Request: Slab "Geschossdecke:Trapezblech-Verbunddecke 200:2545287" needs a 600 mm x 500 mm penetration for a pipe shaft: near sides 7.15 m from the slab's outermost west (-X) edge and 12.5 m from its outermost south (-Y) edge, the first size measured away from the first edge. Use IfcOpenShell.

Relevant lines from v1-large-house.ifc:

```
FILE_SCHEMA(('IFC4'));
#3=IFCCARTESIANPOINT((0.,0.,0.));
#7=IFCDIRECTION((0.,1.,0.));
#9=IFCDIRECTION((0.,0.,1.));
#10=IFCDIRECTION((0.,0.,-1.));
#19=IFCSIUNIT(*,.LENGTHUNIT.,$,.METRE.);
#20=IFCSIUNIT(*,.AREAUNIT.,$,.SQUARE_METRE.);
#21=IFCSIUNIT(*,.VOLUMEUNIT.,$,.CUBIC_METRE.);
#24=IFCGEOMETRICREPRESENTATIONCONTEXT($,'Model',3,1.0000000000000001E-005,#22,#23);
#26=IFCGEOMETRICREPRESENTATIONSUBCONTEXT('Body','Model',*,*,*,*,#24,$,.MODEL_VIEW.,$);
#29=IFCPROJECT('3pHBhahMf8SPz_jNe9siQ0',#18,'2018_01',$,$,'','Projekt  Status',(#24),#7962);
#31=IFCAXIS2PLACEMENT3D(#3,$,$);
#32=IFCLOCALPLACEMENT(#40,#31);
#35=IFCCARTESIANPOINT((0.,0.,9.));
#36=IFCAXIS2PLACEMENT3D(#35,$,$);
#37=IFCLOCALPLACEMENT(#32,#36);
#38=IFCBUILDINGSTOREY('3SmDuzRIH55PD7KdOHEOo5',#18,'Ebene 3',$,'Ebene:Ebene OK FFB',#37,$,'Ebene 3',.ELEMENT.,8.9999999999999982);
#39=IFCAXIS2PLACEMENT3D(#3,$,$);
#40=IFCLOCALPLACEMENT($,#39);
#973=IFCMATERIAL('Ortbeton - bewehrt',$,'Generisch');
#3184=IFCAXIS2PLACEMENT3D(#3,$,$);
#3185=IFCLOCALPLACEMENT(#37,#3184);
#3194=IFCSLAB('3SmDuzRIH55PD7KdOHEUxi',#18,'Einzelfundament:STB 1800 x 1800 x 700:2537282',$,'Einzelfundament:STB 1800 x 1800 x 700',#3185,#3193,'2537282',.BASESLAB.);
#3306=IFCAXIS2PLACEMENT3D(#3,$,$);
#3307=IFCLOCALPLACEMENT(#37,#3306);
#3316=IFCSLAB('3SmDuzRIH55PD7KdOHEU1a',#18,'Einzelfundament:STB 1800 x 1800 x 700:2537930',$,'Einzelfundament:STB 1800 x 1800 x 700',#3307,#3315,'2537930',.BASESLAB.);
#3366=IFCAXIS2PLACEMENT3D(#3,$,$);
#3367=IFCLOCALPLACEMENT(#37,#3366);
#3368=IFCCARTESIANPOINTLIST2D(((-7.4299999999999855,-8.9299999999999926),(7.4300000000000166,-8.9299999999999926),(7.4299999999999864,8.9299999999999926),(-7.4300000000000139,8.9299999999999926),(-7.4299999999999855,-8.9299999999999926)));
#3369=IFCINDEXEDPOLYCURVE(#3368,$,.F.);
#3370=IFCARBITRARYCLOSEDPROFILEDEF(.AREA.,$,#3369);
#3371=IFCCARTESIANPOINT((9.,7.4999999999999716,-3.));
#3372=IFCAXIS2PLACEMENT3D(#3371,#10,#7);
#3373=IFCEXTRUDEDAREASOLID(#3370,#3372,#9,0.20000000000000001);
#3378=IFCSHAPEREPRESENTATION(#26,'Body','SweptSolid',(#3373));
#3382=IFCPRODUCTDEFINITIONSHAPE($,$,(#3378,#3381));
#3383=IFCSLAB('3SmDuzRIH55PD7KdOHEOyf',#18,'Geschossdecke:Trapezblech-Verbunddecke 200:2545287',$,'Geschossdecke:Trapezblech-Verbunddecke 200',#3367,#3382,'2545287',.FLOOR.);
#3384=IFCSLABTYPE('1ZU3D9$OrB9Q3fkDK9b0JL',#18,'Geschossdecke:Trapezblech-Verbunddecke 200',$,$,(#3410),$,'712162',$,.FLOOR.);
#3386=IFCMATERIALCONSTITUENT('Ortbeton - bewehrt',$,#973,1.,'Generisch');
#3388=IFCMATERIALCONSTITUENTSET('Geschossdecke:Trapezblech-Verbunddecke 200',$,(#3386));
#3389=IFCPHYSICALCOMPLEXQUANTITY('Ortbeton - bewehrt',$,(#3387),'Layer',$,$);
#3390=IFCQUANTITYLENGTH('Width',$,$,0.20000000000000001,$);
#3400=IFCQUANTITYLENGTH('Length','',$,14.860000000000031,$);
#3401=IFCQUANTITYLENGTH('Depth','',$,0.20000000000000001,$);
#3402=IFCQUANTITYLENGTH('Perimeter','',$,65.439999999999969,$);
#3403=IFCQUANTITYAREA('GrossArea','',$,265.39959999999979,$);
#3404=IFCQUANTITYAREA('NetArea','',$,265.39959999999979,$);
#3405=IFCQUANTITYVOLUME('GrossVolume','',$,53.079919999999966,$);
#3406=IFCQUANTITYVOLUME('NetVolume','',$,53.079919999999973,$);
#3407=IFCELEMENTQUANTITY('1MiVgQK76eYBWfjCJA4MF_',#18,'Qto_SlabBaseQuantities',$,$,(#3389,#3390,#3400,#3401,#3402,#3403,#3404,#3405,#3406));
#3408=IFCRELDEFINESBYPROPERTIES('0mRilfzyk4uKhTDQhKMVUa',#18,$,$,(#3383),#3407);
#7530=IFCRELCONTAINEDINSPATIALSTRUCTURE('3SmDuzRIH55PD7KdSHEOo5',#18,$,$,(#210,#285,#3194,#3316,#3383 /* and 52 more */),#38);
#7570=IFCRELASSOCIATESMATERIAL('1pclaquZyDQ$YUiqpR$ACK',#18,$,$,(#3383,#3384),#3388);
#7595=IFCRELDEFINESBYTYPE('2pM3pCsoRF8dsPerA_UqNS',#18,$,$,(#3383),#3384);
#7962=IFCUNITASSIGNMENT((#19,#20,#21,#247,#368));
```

```python
import numpy as np
import ifcopenshell
import ifcopenshell.api.feature
import ifcopenshell.api.geometry
import ifcopenshell.api.pset
import ifcopenshell.api.root
import ifcopenshell.geom
import ifcopenshell.util.element
import ifcopenshell.util.placement
import ifcopenshell.util.representation
import ifcopenshell.util.shape
import ifcopenshell.util.unit

model = ifcopenshell.open("v1-large-house.ifc")
unit_scale = ifcopenshell.util.unit.calculate_unit_scale(model)
area_scale = ifcopenshell.util.unit.calculate_unit_scale(model, "AREAUNIT")
volume_scale = ifcopenshell.util.unit.calculate_unit_scale(model, "VOLUMEUNIT")
settings = ifcopenshell.geom.settings()


def volume(element):
    """Net volume in cubic metres, openings subtracted."""
    shape = ifcopenshell.geom.create_shape(settings, element)
    return ifcopenshell.util.shape.get_volume(shape.geometry)


slab = model.by_id(3383)
before = volume(slab)

# Extent in the slab's own axes, in metres. The edges named are its -X and -Y sides.
slab_shape = ifcopenshell.geom.create_shape(settings, slab)
vertices = ifcopenshell.util.shape.get_vertices(slab_shape.geometry)
x_min, y_min, bottom = vertices.min(axis=0)
top = vertices[:, 2].max()

opening = ifcopenshell.api.root.create_entity(model, ifc_class="IfcOpeningElement", name="Pipe shaft opening", predefined_type="OPENING")
context = ifcopenshell.util.representation.get_context(model, "Model", "Body", "MODEL_VIEW")
width, depth = 0.6, 0.5
outline = [(0.0, 0.0), (width, 0.0), (width, depth), (0.0, depth), (0.0, 0.0)]
# Overshoot both faces by 50 mm so the cut is clean.
shape = ifcopenshell.api.geometry.add_slab_representation(
    model, context=context, depth=top - bottom + 0.1, polyline=outline
)
ifcopenshell.api.geometry.assign_representation(model, product=opening, representation=shape)

matrix = ifcopenshell.util.placement.get_local_placement(slab.ObjectPlacement)
matrix[:, 3] = matrix @ np.append(np.array([x_min + 7.15, y_min + 12.5, bottom - 0.05]) / unit_scale, 1.0)
ifcopenshell.api.geometry.edit_object_placement(model, product=opening, matrix=matrix, is_si=False)
ifcopenshell.api.feature.add_feature(model, feature=opening, element=slab)

after = volume(slab)

# Update the slab's stored quantities.
qto = model.by_id(ifcopenshell.util.element.get_pset(slab, "Qto_SlabBaseQuantities", should_inherit=False)["id"])
ifcopenshell.api.pset.edit_qto(model, qto=qto, properties={
    "NetArea": after / (top - bottom) / area_scale,
    "NetVolume": after / volume_scale,
})

print(f"slab volume {before:.3f} -> {after:.3f} m3")

model.write("v1-large-house_edited.ifc")
```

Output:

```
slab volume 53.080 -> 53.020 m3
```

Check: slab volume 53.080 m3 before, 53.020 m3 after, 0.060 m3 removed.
